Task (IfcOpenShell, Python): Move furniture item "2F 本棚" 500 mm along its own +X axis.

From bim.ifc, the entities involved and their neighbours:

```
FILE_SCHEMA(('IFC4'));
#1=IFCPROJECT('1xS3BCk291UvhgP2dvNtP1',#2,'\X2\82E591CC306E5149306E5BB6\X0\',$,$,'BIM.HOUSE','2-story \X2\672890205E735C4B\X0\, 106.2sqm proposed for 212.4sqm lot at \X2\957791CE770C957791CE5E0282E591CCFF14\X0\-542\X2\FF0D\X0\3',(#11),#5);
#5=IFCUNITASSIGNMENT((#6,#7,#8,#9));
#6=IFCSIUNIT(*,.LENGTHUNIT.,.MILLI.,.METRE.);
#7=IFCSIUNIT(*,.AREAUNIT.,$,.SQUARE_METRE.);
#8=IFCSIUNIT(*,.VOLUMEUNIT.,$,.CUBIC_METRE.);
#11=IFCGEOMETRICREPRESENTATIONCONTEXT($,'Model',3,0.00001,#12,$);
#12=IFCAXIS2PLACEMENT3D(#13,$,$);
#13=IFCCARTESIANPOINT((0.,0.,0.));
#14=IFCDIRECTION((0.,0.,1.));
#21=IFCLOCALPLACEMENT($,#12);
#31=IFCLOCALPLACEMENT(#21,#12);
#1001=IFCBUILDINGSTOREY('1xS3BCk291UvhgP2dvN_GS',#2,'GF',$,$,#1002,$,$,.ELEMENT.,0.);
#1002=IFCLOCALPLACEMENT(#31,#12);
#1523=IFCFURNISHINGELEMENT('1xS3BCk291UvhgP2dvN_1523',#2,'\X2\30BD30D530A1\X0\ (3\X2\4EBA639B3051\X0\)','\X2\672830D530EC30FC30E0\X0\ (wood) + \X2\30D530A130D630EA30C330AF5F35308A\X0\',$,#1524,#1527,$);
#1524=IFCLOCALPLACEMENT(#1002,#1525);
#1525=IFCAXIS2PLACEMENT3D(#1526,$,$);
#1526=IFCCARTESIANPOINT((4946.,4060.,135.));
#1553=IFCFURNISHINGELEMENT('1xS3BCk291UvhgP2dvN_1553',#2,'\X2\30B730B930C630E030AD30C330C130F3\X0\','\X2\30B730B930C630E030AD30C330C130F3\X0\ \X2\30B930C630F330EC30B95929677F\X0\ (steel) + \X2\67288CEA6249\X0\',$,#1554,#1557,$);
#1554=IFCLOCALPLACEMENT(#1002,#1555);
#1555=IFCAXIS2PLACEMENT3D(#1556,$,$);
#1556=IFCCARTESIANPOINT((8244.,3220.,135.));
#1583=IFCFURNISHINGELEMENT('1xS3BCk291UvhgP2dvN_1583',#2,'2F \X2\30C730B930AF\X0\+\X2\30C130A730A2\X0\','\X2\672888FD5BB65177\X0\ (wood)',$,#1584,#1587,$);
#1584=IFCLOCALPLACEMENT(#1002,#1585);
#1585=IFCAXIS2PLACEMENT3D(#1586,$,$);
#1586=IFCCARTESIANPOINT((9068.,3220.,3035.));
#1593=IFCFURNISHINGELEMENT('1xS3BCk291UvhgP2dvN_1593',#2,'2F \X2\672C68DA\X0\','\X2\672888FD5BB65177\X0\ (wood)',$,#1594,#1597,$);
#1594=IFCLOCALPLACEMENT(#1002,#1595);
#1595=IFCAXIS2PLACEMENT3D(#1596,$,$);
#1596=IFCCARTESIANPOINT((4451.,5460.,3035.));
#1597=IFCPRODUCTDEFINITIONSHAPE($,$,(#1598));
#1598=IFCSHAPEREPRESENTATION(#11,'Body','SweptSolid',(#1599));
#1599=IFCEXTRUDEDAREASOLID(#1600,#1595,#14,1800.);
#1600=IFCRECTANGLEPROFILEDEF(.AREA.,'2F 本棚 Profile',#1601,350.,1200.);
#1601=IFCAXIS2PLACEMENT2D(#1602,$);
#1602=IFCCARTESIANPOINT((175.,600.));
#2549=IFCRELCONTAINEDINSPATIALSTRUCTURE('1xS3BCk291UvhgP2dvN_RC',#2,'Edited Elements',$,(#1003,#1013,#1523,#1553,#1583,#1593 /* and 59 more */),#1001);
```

```python
import ifcopenshell
import ifcopenshell.api.geometry
import ifcopenshell.util.placement
import ifcopenshell.util.unit

model = ifcopenshell.open("bim.ifc")
unit_scale = ifcopenshell.util.unit.calculate_unit_scale(model)

item = model.by_guid("1xS3BCk291UvhgP2dvN_1593")
matrix = ifcopenshell.util.placement.get_local_placement(item.ObjectPlacement)
matrix[:3, 3] += matrix[:3, 0] * 0.5 / unit_scale
ifcopenshell.api.geometry.edit_object_placement(model, product=item, matrix=matrix, is_si=False)

print(ifcopenshell.util.placement.get_local_placement(item.ObjectPlacement).round(3) + 0.0)

model.write("bim_updated.ifc")
```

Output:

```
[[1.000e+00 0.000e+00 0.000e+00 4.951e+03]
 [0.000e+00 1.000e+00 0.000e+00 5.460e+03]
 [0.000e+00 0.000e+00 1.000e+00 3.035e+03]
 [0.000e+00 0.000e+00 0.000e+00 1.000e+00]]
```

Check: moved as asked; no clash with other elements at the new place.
